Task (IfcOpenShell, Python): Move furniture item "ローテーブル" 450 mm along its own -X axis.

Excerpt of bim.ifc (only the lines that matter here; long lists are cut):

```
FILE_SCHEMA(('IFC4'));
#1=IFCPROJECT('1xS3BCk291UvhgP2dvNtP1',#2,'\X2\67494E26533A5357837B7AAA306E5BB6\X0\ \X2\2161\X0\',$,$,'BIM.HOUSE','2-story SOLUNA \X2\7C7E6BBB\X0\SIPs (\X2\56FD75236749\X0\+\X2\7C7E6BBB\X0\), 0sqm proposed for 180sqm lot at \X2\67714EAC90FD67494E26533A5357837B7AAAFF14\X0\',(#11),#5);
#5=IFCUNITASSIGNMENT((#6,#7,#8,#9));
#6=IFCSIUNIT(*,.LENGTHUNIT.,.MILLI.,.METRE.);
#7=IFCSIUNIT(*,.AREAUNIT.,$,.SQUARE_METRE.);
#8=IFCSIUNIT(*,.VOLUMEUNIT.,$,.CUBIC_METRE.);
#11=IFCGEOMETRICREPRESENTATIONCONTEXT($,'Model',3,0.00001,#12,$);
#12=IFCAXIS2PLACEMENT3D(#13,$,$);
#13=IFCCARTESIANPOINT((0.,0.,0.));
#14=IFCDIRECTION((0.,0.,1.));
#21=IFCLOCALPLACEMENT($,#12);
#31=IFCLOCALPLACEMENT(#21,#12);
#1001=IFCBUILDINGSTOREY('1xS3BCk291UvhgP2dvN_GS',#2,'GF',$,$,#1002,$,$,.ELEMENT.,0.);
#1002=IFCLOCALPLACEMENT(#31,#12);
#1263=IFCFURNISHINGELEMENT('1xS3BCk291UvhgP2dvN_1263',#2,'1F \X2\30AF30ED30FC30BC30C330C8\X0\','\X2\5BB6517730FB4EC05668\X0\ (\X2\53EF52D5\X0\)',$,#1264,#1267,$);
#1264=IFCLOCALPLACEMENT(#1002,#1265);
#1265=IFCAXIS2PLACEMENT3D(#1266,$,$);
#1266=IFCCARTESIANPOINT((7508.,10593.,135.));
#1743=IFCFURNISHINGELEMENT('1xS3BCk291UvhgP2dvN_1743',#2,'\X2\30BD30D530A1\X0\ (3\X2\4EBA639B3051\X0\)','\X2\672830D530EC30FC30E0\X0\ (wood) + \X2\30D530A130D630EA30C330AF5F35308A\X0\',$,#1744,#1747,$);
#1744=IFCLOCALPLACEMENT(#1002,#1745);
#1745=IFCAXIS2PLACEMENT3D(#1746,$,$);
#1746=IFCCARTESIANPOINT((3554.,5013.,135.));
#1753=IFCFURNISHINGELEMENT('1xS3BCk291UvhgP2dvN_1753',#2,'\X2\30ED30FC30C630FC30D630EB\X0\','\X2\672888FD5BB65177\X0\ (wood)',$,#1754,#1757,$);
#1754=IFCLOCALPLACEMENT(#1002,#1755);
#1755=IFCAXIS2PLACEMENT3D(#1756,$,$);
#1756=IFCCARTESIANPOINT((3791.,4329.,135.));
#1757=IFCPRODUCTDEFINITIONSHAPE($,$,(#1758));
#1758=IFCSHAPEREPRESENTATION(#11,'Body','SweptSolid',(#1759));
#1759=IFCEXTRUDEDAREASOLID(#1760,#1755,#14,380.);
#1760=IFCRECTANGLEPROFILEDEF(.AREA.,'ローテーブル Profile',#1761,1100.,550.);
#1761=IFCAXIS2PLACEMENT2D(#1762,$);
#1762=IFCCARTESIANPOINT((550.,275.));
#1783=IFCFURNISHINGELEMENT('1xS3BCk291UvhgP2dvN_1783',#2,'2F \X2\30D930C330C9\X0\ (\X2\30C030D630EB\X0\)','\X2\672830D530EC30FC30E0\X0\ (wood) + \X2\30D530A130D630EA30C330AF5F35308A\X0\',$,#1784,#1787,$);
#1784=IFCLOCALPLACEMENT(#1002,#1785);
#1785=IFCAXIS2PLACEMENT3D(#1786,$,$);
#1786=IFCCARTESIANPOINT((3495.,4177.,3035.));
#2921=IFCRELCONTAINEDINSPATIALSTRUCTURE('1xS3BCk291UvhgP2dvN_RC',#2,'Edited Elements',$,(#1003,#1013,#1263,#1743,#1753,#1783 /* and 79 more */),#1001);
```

```python
import ifcopenshell
import ifcopenshell.api.geometry
import ifcopenshell.util.placement

model = ifcopenshell.open("bim.ifc")

item = model.by_guid("1xS3BCk291UvhgP2dvN_1753")
matrix = ifcopenshell.util.placement.get_local_placement(item.ObjectPlacement)
matrix[:3, 3] -= matrix[:3, 0] * 450.0
ifcopenshell.api.geometry.edit_object_placement(model, product=item, matrix=matrix, is_si=False)

print(ifcopenshell.util.placement.get_local_placement(item.ObjectPlacement).round(3) + 0.0)

model.write("bim_edited.ifc")
```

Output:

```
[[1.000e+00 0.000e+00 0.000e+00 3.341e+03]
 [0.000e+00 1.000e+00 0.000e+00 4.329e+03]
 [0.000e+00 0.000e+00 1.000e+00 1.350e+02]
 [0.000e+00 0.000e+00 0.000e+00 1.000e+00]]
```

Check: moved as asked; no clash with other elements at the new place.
